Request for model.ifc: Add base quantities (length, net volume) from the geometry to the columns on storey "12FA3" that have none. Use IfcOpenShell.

First a look at what the model holds.

```python
import ifcopenshell
import ifcopenshell.util.element
import ifcopenshell.util.unit

model = ifcopenshell.open("model.ifc")
print(model.schema)
for unit_type in ("LENGTHUNIT", "AREAUNIT", "VOLUMEUNIT"):
    print(unit_type, ifcopenshell.util.unit.calculate_unit_scale(model, unit_type))
storey = next(s for s in model.by_type("IfcBuildingStorey") if s.Name == "12FA3")
columns = [e for e in ifcopenshell.util.element.get_decomposition(storey) if e.is_a("IfcColumn")]
for e in sorted(columns, key=lambda e: e.id()):
    print(e.id(), e.is_a(), e.Name, list(ifcopenshell.util.element.get_psets(e, qtos_only=True)), sep=" | ")
```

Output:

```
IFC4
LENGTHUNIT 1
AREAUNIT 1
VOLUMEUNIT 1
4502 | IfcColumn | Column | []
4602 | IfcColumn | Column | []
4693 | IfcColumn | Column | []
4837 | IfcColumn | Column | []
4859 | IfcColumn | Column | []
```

```python
import ifcopenshell
import ifcopenshell.api.pset
import ifcopenshell.geom
import ifcopenshell.util.element
import ifcopenshell.util.shape
import ifcopenshell.util.unit

model = ifcopenshell.open("model.ifc")
unit_scale = ifcopenshell.util.unit.calculate_unit_scale(model)
volume_scale = ifcopenshell.util.unit.calculate_unit_scale(model, "VOLUMEUNIT")
settings = ifcopenshell.geom.settings()

storey = next(s for s in model.by_type("IfcBuildingStorey") if s.Name == "12FA3")
columns = [e for e in ifcopenshell.util.element.get_decomposition(storey) if e.is_a("IfcColumn")]

for e in sorted(columns, key=lambda e: e.id()):
    if ifcopenshell.util.element.get_psets(e, qtos_only=True, should_inherit=False):
        continue
    # Geometry comes back in metres, in the element's own axes.
    shape = ifcopenshell.geom.create_shape(settings, e)
    values = {
        "Length": ifcopenshell.util.shape.get_z(shape.geometry) / unit_scale,
        "NetVolume": ifcopenshell.util.shape.get_volume(shape.geometry) / volume_scale,
    }
    qto = ifcopenshell.api.pset.add_qto(model, product=e, name="Qto_ColumnBaseQuantities")
    ifcopenshell.api.pset.edit_qto(model, qto=qto, properties=values)
    print(e.id(), {k: round(v, 3) for k, v in values.items()})

model.write("model_updated.ifc")
```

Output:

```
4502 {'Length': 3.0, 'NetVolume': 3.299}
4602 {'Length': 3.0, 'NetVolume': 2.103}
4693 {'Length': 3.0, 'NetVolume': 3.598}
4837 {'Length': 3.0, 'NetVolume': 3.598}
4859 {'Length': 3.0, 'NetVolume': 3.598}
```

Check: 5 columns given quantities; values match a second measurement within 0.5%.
